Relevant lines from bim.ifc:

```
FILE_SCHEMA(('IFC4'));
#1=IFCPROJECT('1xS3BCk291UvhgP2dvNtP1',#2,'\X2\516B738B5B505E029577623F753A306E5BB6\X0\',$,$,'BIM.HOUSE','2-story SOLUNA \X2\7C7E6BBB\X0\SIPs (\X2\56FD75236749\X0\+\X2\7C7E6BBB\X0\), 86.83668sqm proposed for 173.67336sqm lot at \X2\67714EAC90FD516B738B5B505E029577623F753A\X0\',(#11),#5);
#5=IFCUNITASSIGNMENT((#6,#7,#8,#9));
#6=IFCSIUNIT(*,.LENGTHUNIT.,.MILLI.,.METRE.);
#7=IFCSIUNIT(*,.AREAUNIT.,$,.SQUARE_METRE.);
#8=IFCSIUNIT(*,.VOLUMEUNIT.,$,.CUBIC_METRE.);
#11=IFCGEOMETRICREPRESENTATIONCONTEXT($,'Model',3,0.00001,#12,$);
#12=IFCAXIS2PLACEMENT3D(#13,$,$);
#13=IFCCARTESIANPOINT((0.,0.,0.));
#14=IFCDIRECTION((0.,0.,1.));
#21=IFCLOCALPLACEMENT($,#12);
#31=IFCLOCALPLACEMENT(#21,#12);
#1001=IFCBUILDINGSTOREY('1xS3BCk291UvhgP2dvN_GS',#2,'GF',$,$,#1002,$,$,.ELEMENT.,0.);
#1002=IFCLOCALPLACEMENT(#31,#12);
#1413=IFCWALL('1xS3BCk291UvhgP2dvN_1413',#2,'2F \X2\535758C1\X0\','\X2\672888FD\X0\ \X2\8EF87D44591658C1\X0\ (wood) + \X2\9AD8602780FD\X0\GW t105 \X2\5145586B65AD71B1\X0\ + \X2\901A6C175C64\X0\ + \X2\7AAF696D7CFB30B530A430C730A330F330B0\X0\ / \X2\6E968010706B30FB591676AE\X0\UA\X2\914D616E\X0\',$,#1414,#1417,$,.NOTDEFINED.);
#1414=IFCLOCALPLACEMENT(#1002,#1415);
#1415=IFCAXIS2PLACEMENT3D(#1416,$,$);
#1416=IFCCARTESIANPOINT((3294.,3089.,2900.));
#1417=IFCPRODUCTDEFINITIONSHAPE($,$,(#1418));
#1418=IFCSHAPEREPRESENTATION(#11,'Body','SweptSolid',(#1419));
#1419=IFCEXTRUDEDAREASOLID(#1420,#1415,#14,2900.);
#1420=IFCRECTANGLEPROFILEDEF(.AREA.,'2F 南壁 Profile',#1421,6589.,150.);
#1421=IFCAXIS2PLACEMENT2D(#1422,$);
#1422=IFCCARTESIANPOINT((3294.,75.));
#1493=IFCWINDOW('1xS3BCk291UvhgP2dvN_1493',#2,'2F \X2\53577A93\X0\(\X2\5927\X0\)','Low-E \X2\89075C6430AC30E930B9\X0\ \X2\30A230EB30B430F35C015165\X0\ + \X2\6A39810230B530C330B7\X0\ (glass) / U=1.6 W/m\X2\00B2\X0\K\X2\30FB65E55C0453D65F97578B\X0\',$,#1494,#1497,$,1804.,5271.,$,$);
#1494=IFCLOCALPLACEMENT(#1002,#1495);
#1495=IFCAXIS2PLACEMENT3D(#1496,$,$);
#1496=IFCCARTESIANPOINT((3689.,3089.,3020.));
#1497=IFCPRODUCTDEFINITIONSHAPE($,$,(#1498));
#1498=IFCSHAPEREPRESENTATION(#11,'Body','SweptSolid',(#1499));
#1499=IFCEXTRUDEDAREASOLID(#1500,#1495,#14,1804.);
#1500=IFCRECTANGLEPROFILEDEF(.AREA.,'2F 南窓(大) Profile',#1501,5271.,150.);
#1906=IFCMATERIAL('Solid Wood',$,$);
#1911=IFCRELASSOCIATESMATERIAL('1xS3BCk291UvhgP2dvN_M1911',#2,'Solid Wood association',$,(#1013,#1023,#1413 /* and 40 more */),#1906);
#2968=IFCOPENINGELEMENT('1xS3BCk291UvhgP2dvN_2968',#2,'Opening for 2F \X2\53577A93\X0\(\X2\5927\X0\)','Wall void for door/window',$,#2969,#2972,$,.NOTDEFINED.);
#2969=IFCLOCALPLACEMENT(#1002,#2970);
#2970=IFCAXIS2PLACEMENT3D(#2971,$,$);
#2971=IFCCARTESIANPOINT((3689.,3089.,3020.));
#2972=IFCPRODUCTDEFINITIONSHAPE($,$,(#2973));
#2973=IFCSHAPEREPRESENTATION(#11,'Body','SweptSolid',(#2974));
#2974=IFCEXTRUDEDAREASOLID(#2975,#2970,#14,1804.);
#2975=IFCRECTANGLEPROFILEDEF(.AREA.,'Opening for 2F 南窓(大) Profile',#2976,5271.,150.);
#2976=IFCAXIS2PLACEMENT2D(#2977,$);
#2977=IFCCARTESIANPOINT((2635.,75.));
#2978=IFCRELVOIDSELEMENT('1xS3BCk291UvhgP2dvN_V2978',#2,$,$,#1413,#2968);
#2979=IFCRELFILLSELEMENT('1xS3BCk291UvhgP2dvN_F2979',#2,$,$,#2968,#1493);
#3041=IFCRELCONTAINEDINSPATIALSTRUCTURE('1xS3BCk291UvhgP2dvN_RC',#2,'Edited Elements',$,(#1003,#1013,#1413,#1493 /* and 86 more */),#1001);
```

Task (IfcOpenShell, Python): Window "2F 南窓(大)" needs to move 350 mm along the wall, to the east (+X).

```python
import ifcopenshell
import ifcopenshell.api.geometry
import ifcopenshell.util.placement
import ifcopenshell.util.unit

model = ifcopenshell.open("bim.ifc")
unit_scale = ifcopenshell.util.unit.calculate_unit_scale(model)

window = model.by_guid("1xS3BCk291UvhgP2dvN_1493")
opening = window.FillsVoids[0].RelatingOpeningElement
wall = opening.VoidsElements[0].RelatingBuildingElement

wall_matrix = ifcopenshell.util.placement.get_local_placement(wall.ObjectPlacement)
shift = wall_matrix[:3, 0] * 0.35 / unit_scale
before = ifcopenshell.util.placement.get_local_placement(window.ObjectPlacement)[:3, 3].copy()

# The window is not placed relative to its opening, so move both.
for product in (opening, window):
    matrix = ifcopenshell.util.placement.get_local_placement(product.ObjectPlacement)
    matrix[:3, 3] += shift
    ifcopenshell.api.geometry.edit_object_placement(model, product=product, matrix=matrix, is_si=False)

after = ifcopenshell.util.placement.get_local_placement(window.ObjectPlacement)[:3, 3]
print("window moved by", (after - before).round(3) + 0.0)

model.write("bim_updated.ifc")
```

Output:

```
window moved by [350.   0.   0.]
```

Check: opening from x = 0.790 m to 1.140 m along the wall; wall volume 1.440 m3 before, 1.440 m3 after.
